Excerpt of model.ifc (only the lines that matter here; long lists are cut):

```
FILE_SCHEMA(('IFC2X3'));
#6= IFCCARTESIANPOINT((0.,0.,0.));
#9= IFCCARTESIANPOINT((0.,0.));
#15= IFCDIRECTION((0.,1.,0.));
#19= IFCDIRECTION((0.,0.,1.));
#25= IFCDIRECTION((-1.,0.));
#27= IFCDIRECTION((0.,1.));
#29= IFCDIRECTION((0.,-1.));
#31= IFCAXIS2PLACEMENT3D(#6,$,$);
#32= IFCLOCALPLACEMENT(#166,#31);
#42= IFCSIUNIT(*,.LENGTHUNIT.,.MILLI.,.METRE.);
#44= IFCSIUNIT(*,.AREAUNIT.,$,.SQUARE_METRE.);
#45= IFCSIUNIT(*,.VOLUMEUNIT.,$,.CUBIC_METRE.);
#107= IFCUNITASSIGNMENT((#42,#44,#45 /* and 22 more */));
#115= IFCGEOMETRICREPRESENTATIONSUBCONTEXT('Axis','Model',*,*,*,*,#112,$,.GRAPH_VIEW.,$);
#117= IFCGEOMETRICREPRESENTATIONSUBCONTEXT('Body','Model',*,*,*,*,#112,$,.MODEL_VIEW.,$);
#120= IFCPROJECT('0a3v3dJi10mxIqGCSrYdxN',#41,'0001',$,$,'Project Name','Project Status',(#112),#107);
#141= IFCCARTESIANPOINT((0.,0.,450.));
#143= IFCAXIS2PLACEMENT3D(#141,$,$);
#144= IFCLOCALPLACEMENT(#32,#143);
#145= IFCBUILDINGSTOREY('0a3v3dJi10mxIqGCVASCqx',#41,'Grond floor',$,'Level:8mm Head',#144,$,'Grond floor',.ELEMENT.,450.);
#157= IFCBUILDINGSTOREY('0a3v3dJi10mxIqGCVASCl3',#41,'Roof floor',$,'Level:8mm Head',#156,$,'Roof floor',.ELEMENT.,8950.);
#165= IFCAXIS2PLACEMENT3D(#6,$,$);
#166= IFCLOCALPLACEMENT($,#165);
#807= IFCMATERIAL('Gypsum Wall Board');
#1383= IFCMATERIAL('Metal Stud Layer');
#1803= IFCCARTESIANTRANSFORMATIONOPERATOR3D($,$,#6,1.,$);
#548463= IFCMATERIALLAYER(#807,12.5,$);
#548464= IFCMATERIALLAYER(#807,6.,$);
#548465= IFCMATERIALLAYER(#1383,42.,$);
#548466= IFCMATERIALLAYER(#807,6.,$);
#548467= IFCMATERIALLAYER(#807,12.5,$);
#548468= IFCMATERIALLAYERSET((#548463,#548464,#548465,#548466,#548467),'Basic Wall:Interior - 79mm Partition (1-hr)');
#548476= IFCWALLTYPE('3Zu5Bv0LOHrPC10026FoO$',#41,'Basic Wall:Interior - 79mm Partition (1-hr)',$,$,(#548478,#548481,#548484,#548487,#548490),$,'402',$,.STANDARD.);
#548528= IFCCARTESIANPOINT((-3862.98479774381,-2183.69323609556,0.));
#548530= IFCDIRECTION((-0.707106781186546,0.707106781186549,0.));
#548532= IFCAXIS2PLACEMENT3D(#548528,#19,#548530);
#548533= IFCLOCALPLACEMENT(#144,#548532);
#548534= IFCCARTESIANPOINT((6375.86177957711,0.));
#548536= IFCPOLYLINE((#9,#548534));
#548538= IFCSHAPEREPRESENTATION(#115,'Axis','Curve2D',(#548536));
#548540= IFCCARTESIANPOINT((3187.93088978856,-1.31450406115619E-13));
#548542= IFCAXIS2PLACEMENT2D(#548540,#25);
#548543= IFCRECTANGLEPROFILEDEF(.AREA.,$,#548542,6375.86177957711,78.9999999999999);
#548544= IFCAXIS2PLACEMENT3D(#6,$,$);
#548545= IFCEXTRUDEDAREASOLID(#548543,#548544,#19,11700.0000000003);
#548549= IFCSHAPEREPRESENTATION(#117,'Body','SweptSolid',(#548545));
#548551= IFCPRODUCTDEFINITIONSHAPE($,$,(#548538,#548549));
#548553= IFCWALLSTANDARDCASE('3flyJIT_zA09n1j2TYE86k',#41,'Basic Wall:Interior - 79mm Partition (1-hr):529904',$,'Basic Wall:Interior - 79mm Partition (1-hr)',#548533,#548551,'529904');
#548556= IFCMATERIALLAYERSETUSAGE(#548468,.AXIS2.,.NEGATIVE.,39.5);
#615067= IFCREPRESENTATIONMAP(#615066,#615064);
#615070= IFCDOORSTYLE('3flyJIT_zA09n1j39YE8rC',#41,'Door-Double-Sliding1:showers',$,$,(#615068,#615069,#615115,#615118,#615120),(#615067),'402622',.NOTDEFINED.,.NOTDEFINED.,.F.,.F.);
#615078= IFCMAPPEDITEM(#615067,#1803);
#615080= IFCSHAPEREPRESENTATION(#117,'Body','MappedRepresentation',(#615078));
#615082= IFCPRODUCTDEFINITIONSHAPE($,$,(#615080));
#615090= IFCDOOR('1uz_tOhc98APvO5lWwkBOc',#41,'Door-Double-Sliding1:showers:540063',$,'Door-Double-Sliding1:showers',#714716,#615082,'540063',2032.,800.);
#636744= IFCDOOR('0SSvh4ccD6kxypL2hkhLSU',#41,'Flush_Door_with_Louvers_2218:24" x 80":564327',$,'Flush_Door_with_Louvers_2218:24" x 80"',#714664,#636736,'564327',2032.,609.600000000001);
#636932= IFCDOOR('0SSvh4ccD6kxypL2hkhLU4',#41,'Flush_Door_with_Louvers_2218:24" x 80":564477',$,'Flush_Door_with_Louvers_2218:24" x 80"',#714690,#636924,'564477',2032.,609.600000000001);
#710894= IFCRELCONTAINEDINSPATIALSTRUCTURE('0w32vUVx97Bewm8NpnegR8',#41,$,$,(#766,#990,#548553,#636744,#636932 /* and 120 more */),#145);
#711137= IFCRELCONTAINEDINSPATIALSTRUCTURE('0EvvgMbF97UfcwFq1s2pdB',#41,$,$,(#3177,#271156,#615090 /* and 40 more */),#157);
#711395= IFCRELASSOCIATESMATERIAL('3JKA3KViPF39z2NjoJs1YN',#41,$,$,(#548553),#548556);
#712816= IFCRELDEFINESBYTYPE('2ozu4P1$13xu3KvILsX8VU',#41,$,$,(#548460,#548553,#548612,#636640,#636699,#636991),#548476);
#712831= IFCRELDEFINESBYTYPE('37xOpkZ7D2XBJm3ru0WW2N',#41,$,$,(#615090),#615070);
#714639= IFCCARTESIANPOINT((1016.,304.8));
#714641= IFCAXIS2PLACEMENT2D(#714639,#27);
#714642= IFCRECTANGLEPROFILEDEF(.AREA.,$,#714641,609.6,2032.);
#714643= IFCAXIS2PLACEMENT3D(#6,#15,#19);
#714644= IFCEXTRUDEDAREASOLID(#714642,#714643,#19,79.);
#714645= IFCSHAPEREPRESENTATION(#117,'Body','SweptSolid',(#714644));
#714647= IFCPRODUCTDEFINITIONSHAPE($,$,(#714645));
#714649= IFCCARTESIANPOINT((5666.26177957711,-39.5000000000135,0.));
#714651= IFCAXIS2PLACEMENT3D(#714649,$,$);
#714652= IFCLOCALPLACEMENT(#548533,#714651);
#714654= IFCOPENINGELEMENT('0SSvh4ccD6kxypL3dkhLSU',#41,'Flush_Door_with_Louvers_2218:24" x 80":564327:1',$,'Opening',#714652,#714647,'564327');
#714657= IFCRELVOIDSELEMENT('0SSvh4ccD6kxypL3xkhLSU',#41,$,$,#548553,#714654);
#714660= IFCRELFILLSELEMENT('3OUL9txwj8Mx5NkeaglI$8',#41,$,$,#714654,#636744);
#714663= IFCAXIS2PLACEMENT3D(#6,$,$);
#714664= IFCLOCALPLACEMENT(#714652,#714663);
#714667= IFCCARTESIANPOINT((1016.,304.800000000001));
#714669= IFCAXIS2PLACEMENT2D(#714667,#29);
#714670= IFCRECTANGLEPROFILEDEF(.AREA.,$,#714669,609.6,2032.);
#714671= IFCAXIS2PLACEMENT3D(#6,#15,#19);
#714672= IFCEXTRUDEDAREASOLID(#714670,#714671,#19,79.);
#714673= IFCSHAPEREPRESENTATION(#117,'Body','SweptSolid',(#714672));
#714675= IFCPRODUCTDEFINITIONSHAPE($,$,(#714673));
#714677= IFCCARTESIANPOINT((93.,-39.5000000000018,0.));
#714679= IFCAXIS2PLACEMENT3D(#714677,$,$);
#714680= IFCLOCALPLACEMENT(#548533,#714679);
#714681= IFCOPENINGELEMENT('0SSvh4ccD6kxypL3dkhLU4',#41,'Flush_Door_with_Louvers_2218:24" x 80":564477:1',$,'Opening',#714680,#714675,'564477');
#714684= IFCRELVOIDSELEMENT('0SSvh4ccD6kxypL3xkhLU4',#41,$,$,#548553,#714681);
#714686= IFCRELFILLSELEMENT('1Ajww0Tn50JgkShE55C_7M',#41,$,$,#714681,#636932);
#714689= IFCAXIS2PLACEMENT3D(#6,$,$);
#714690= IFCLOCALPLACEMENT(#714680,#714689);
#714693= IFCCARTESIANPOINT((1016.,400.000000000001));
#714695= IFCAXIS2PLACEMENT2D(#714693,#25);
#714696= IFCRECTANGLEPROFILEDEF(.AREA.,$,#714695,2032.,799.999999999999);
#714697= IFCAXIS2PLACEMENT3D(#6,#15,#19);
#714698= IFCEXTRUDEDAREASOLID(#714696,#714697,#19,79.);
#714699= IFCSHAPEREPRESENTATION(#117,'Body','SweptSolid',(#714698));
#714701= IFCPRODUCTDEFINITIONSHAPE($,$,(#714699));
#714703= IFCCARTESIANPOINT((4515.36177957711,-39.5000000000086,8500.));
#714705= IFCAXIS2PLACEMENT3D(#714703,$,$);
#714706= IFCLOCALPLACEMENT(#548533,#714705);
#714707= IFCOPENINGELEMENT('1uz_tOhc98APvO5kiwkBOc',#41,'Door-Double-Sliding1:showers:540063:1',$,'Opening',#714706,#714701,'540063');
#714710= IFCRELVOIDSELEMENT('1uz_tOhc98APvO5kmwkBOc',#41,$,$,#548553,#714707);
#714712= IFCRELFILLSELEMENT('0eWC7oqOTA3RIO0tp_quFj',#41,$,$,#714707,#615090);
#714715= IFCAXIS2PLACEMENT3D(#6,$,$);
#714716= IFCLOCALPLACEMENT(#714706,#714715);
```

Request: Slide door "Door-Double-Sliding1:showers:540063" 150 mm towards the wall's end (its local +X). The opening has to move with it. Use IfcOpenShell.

```python
import ifcopenshell
import ifcopenshell.api.geometry
import ifcopenshell.util.placement
import ifcopenshell.util.unit

model = ifcopenshell.open("model.ifc")
unit_scale = ifcopenshell.util.unit.calculate_unit_scale(model)

door = model.by_id(615090)
opening = door.FillsVoids[0].RelatingOpeningElement
wall = opening.VoidsElements[0].RelatingBuildingElement

wall_matrix = ifcopenshell.util.placement.get_local_placement(wall.ObjectPlacement)
shift = wall_matrix[:3, 0] * 0.15 / unit_scale
before = ifcopenshell.util.placement.get_local_placement(door.ObjectPlacement)[:3, 3].copy()

# The door is placed relative to its opening, so it follows when the opening moves.
matrix = ifcopenshell.util.placement.get_local_placement(opening.ObjectPlacement)
matrix[:3, 3] += shift
ifcopenshell.api.geometry.edit_object_placement(
    model, product=opening, matrix=matrix, is_si=False, should_transform_children=True
)

after = ifcopenshell.util.placement.get_local_placement(door.ObjectPlacement)[:3, 3]
print("door moved by", (after - before).round(3) + 0.0)

model.write("model-out.ifc")
```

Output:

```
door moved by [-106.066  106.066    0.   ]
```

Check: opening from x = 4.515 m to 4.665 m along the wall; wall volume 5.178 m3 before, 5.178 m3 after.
